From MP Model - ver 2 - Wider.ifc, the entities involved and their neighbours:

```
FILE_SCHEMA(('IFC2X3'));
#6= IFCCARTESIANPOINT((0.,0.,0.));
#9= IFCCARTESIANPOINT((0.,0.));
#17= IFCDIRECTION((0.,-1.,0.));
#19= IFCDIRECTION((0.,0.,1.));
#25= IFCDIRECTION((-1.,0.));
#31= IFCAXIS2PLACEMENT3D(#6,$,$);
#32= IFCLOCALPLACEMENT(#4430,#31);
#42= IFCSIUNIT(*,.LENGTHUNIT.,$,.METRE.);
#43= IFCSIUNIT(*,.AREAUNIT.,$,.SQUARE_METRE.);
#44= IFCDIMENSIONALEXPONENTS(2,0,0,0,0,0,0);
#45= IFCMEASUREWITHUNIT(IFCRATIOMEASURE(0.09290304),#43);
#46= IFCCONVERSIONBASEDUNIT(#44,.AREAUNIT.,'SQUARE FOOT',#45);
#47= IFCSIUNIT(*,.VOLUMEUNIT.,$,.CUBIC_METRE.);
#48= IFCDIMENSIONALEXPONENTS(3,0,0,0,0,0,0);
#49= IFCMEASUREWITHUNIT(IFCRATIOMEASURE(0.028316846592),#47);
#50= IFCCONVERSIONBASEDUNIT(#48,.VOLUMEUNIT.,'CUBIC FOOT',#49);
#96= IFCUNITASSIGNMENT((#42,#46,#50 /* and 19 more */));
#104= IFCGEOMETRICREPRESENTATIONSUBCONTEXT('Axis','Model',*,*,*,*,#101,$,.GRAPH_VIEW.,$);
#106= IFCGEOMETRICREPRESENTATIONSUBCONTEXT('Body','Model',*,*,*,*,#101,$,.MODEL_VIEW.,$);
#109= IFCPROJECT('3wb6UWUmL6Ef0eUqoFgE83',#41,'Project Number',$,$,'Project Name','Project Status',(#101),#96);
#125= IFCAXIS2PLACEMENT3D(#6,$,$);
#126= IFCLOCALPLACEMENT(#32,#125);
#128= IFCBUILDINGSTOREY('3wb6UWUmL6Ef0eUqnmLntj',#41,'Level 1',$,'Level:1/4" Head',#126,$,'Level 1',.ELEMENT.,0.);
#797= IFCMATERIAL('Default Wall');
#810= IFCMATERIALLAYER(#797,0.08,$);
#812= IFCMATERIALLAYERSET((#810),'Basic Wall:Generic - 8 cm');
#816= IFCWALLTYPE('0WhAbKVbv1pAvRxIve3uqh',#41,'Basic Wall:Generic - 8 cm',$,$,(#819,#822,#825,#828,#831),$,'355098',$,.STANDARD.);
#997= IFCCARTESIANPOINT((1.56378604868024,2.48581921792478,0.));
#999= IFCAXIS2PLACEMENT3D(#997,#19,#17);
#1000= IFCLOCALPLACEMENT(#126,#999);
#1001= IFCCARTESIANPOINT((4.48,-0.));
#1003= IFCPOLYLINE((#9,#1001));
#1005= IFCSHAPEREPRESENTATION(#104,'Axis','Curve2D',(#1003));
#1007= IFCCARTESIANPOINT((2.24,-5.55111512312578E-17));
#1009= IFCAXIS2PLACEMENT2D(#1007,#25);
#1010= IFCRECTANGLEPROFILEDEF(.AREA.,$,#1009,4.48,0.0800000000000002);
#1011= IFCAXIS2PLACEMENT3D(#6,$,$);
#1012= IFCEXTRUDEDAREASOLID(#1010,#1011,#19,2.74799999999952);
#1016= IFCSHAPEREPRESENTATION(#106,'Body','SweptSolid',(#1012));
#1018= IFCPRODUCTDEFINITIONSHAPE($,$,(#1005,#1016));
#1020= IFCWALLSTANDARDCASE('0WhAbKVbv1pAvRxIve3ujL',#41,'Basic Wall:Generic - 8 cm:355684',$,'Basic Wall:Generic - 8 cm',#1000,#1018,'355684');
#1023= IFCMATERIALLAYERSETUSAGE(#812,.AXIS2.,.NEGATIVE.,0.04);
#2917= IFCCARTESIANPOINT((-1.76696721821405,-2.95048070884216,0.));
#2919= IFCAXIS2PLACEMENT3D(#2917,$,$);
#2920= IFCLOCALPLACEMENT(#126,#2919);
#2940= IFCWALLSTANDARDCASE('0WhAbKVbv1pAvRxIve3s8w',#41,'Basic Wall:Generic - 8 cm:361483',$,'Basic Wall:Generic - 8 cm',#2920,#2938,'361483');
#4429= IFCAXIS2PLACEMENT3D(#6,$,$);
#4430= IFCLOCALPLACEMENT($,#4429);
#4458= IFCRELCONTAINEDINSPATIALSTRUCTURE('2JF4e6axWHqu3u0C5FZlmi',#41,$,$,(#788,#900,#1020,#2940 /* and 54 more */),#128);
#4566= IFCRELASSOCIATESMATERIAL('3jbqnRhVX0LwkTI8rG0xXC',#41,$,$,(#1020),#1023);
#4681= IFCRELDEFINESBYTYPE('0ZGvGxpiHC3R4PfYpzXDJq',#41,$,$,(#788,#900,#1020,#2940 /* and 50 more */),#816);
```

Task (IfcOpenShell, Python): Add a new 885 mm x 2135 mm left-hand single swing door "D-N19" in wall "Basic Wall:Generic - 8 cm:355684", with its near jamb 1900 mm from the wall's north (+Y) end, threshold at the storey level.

```python
import numpy as np
import ifcopenshell
import ifcopenshell.api.feature
import ifcopenshell.api.geometry
import ifcopenshell.api.root
import ifcopenshell.api.spatial
import ifcopenshell.api.type
import ifcopenshell.geom
import ifcopenshell.util.element
import ifcopenshell.util.placement
import ifcopenshell.util.representation
import ifcopenshell.util.shape
import ifcopenshell.util.unit

model = ifcopenshell.open("MP Model - ver 2 - Wider.ifc")
unit_scale = ifcopenshell.util.unit.calculate_unit_scale(model)
settings = ifcopenshell.geom.settings()


def volume(element):
    """Net volume in cubic metres, openings subtracted."""
    shape = ifcopenshell.geom.create_shape(settings, element)
    return ifcopenshell.util.shape.get_volume(shape.geometry)


wall = model.by_guid("0WhAbKVbv1pAvRxIve3ujL")
storey = ifcopenshell.util.element.get_container(wall, ifc_class="IfcBuildingStorey")
context = ifcopenshell.util.representation.get_context(model, "Model", "Body", "MODEL_VIEW")
before = volume(wall)

width, height, from_end, sill = 0.885, 2.135, 1.9, 0.0  # metres

# The wall runs along its own X axis, and the end named is its -X end.
wall_shape = ifcopenshell.geom.create_shape(settings, wall)
x, y, z = ifcopenshell.util.shape.get_vertices(wall_shape.geometry).T
start = x.min() + from_end
face, thickness = float(y.min()), float(y.max() - y.min())
wall_matrix = ifcopenshell.util.placement.get_local_placement(wall.ObjectPlacement)
level = ifcopenshell.util.placement.get_local_placement(storey.ObjectPlacement)[2, 3]


def in_wall(x, y):
    """Placement at x, y metres in the wall's axes, at sill height."""
    matrix = wall_matrix.copy()
    matrix[:, 3] = wall_matrix @ np.array([x / unit_scale, y / unit_scale, 0.0, 1.0])
    matrix[2, 3] = level + sill / unit_scale
    return matrix


# Opening: a box that overshoots both wall faces by 50 mm.
opening = ifcopenshell.api.root.create_entity(model, ifc_class="IfcOpeningElement")
box = ifcopenshell.api.geometry.add_wall_representation(
    model, context=context, length=width, height=height, thickness=thickness + 0.1
)
ifcopenshell.api.geometry.assign_representation(model, product=opening, representation=box)
ifcopenshell.api.geometry.edit_object_placement(model, product=opening, matrix=in_wall(start, face - 0.05), is_si=False)
ifcopenshell.api.feature.add_feature(model, feature=opening, element=wall)

door = ifcopenshell.api.root.create_entity(model, ifc_class="IfcDoor", name="D-N19")
door.OverallWidth, door.OverallHeight = width / unit_scale, height / unit_scale
body = ifcopenshell.api.geometry.add_door_representation(
    model,
    context=context,
    overall_width=door.OverallWidth,
    overall_height=door.OverallHeight,
    operation_type="SINGLE_SWING_LEFT",
    lining_properties={"LiningDepth": thickness / unit_scale, "ThresholdDepth": thickness / unit_scale},
)
ifcopenshell.api.geometry.assign_representation(model, product=door, representation=body)
ifcopenshell.api.spatial.assign_container(model, products=[door], relating_structure=storey)
fills = ifcopenshell.api.feature.add_filling(model, opening=opening, element=door)
fills.OwnerHistory = door.OwnerHistory  # required in IFC2X3

# IFC2X3 keeps the operation on the door style.
style = ifcopenshell.api.root.create_entity(model, ifc_class="IfcDoorStyle", name="D-N19")
style.OperationType, style.ConstructionType = "SINGLE_SWING_LEFT", "NOTDEFINED"
style.ParameterTakesPrecedence = style.Sizeable = False
ifcopenshell.api.type.assign_type(model, related_objects=[door], relating_type=style)

# The lining spans the wall, so the door starts at the wall face.
ifcopenshell.api.geometry.edit_object_placement(model, product=door, matrix=in_wall(start, face), is_si=False)

after = volume(wall)

print(f"wall volume {before:.3f} -> {after:.3f} m3")

model.write("MP Model - ver 2 - Wider_rev.ifc")
```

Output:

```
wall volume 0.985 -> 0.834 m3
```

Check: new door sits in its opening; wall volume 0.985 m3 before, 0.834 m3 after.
